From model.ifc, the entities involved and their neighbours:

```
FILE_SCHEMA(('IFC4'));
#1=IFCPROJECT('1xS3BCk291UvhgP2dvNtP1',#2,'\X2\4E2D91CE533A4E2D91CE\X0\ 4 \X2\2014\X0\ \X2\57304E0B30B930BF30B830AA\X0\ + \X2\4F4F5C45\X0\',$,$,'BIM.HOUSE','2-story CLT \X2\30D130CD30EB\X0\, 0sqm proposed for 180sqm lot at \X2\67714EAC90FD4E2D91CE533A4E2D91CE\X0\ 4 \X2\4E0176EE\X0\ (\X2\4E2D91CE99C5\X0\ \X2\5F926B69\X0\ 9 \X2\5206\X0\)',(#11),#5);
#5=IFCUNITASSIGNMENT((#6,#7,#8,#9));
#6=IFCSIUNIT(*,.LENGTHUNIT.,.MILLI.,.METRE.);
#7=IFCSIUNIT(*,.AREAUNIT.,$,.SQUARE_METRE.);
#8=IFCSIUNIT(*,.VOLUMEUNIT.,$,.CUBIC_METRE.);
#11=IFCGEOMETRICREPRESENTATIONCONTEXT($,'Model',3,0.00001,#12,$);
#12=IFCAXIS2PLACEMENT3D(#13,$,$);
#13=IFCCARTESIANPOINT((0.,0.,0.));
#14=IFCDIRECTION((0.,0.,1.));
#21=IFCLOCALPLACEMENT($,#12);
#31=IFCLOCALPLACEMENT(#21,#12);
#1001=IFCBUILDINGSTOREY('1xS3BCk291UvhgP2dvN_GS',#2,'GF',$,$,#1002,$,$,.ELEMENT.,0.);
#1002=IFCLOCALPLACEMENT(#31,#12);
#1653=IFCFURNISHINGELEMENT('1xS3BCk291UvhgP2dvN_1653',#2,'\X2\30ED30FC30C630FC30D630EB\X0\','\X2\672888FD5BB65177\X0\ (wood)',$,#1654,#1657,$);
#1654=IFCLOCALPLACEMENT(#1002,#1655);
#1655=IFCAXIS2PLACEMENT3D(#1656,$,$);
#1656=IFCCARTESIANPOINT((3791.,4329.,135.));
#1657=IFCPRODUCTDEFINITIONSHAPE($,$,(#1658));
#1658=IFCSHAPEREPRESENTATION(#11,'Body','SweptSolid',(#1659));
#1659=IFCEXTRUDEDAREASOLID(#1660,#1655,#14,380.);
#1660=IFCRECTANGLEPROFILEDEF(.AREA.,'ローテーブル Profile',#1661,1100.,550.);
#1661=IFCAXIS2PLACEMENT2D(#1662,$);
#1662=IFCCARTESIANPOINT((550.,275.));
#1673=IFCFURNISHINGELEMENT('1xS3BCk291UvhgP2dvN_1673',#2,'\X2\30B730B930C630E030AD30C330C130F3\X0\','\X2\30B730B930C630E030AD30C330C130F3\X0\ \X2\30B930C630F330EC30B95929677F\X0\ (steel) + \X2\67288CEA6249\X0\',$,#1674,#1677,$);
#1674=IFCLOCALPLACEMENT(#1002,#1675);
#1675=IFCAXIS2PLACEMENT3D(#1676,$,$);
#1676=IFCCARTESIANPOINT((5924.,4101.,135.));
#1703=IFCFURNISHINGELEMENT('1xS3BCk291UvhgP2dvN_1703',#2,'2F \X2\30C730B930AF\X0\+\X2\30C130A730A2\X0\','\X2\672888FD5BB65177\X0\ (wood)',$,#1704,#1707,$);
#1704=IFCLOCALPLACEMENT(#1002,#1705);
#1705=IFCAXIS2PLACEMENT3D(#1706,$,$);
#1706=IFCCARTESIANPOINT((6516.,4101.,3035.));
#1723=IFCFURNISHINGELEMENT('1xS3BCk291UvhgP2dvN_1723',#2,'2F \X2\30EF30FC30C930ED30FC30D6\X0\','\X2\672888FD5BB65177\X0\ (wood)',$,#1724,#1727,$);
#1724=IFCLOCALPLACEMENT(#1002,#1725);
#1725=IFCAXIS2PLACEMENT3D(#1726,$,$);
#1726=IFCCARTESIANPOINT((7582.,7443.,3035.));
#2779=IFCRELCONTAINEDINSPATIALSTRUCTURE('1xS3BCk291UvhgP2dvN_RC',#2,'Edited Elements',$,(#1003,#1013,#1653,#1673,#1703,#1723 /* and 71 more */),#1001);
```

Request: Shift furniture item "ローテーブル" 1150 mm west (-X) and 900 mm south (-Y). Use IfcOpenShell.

```python
import ifcopenshell
import ifcopenshell.api.geometry
import ifcopenshell.util.placement

model = ifcopenshell.open("model.ifc")

item = model.by_guid("1xS3BCk291UvhgP2dvN_1653")
matrix = ifcopenshell.util.placement.get_local_placement(item.ObjectPlacement)
matrix[0, 3] -= 1150.0
matrix[1, 3] -= 900.0
ifcopenshell.api.geometry.edit_object_placement(model, product=item, matrix=matrix, is_si=False)

print(ifcopenshell.util.placement.get_local_placement(item.ObjectPlacement).round(3) + 0.0)

model.write("model_rev.ifc")
```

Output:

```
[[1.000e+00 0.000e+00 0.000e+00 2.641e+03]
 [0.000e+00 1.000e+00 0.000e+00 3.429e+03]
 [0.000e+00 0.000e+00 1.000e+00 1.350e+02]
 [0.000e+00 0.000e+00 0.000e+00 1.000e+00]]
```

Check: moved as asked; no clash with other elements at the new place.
